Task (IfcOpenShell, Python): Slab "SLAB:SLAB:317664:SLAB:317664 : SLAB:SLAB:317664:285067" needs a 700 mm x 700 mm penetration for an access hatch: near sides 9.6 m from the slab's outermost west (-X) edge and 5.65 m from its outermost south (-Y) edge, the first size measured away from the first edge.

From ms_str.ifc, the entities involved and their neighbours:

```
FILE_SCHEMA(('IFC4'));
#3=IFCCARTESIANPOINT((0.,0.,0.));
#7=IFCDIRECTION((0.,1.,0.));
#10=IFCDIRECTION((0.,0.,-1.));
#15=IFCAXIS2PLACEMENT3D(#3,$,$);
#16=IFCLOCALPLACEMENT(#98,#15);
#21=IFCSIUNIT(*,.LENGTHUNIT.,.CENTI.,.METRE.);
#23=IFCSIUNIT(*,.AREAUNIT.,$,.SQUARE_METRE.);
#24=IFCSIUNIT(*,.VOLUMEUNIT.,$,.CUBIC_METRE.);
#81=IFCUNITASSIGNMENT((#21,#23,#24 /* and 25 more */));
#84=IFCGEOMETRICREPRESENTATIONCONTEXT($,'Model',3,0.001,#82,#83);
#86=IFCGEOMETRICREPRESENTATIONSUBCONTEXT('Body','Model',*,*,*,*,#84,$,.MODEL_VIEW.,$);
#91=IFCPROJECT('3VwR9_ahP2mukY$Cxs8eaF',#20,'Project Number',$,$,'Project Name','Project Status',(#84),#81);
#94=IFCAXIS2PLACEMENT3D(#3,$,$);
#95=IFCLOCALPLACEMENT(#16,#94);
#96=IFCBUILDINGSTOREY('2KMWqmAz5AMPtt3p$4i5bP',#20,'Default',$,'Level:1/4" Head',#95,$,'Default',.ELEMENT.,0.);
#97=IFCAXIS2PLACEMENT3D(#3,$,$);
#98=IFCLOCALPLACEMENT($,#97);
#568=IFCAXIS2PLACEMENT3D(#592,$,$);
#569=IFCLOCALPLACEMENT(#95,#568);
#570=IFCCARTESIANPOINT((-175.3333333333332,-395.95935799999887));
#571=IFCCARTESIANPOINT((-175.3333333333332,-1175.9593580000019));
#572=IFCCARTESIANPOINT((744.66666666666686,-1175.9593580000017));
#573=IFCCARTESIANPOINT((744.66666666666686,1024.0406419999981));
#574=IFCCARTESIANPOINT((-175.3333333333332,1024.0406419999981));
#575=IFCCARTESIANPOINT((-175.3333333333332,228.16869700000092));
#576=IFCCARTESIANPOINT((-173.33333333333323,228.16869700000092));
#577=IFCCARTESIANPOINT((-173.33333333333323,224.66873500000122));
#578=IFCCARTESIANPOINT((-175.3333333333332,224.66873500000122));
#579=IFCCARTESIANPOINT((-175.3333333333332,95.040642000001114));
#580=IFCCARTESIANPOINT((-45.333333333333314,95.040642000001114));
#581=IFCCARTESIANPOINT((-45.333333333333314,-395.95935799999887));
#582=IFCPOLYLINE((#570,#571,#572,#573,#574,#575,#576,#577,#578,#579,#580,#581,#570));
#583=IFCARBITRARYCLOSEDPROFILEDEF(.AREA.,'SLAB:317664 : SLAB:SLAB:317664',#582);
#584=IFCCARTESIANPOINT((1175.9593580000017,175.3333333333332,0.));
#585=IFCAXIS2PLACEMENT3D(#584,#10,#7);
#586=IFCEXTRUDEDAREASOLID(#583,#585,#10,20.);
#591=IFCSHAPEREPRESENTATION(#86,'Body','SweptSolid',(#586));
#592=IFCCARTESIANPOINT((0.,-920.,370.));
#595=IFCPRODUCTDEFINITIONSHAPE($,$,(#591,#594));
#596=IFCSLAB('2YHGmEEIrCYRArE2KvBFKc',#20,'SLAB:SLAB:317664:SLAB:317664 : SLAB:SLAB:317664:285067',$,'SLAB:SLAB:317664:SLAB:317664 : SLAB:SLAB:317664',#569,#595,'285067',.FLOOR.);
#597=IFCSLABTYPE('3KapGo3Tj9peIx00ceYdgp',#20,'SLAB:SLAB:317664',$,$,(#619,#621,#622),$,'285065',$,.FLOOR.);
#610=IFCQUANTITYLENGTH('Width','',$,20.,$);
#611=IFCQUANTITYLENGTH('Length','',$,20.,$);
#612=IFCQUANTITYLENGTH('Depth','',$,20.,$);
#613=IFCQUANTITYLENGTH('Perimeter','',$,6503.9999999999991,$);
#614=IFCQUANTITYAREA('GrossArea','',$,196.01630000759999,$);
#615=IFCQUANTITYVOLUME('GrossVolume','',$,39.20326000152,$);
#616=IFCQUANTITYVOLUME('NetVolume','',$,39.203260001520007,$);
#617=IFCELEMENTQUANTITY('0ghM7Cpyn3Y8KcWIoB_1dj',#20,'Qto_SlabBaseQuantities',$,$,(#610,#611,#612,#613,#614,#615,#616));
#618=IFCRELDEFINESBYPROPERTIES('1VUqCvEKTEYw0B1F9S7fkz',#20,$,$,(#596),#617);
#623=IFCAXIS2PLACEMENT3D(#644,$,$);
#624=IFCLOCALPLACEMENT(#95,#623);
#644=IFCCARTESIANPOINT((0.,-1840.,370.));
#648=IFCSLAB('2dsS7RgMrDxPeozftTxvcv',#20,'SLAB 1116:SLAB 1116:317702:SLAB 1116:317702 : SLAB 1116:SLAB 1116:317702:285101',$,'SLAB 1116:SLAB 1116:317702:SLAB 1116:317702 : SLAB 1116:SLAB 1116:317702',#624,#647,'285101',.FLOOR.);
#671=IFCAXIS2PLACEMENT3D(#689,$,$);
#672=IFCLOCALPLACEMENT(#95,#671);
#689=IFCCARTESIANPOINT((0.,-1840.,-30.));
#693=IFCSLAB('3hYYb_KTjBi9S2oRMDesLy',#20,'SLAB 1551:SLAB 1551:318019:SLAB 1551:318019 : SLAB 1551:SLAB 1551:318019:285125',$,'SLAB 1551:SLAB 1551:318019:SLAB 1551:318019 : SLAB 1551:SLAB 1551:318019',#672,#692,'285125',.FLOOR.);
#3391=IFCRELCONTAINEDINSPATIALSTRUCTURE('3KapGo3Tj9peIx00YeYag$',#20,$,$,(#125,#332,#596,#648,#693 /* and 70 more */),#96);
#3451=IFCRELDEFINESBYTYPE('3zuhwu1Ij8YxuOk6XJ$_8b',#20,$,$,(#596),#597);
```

```python
import numpy as np
import ifcopenshell
import ifcopenshell.api.feature
import ifcopenshell.api.geometry
import ifcopenshell.api.pset
import ifcopenshell.api.root
import ifcopenshell.geom
import ifcopenshell.util.element
import ifcopenshell.util.placement
import ifcopenshell.util.representation
import ifcopenshell.util.shape
import ifcopenshell.util.unit

model = ifcopenshell.open("ms_str.ifc")
unit_scale = ifcopenshell.util.unit.calculate_unit_scale(model)
volume_scale = ifcopenshell.util.unit.calculate_unit_scale(model, "VOLUMEUNIT")
settings = ifcopenshell.geom.settings()


def volume(element):
    """Net volume in cubic metres, openings subtracted."""
    shape = ifcopenshell.geom.create_shape(settings, element)
    return ifcopenshell.util.shape.get_volume(shape.geometry)


slab = model.by_id(596)
before = volume(slab)

# Extent in the slab's own axes, in metres. The edges named are its -X and -Y sides.
slab_shape = ifcopenshell.geom.create_shape(settings, slab)
vertices = ifcopenshell.util.shape.get_vertices(slab_shape.geometry)
x_min, y_min, bottom = vertices.min(axis=0)
top = vertices[:, 2].max()

opening = ifcopenshell.api.root.create_entity(model, ifc_class="IfcOpeningElement", name="Access hatch opening", predefined_type="OPENING")
context = ifcopenshell.util.representation.get_context(model, "Model", "Body", "MODEL_VIEW")
width, depth = 0.7, 0.7
outline = [(0.0, 0.0), (width, 0.0), (width, depth), (0.0, depth), (0.0, 0.0)]
# Overshoot both faces by 50 mm so the cut is clean.
shape = ifcopenshell.api.geometry.add_slab_representation(
    model, context=context, depth=top - bottom + 0.1, polyline=outline
)
ifcopenshell.api.geometry.assign_representation(model, product=opening, representation=shape)

matrix = ifcopenshell.util.placement.get_local_placement(slab.ObjectPlacement)
matrix[:, 3] = matrix @ np.append(np.array([x_min + 9.6, y_min + 5.65, bottom - 0.05]) / unit_scale, 1.0)
ifcopenshell.api.geometry.edit_object_placement(model, product=opening, matrix=matrix, is_si=False)
ifcopenshell.api.feature.add_feature(model, feature=opening, element=slab)

after = volume(slab)

# Update the slab's stored quantities.
qto = model.by_id(ifcopenshell.util.element.get_pset(slab, "Qto_SlabBaseQuantities", should_inherit=False)["id"])
ifcopenshell.api.pset.edit_qto(model, qto=qto, properties={"NetVolume": after / volume_scale})

print(f"slab volume {before:.3f} -> {after:.3f} m3")

model.write("ms_str-out.ifc")
```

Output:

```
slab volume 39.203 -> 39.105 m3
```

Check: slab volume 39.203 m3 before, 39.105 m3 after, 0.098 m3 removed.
